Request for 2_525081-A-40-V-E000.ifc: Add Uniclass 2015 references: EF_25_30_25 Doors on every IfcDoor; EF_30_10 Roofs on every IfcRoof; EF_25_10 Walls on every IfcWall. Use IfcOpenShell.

First a look at what the model holds.

```python
import ifcopenshell

model = ifcopenshell.open("2_525081-A-40-V-E000.ifc")
print(model.schema)
print("classifications:", [c.Name for c in model.by_type("IfcClassification")])
for ifc_class in ("IfcDoor", "IfcRoof", "IfcStair", "IfcWall", "IfcWindow"):
    print(ifc_class, len(model.by_type(ifc_class)))
```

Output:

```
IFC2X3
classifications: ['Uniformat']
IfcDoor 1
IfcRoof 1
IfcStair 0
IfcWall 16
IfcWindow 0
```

```python
import ifcopenshell
import ifcopenshell.api.classification

model = ifcopenshell.open("2_525081-A-40-V-E000.ifc")

# IFC2X3 requires Source and Edition and has no link from the project to the system.
system = model.create_entity("IfcClassification", Source="NBS", Edition="2015", Name="Uniclass 2015")

codes = {
    "IfcDoor": ("EF_25_30_25", "Doors"),
    "IfcRoof": ("EF_30_10", "Roofs"),
    "IfcWall": ("EF_25_10", "Walls"),
}
for ifc_class, (code, name) in codes.items():
    products = model.by_type(ifc_class)
    ifcopenshell.api.classification.add_reference(
        model, products=products, classification=system, identification=code, name=name
    )
    print(code, len(products))

model.write("2_525081-A-40-V-E000_updated.ifc")
```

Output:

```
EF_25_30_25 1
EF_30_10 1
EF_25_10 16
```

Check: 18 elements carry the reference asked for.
